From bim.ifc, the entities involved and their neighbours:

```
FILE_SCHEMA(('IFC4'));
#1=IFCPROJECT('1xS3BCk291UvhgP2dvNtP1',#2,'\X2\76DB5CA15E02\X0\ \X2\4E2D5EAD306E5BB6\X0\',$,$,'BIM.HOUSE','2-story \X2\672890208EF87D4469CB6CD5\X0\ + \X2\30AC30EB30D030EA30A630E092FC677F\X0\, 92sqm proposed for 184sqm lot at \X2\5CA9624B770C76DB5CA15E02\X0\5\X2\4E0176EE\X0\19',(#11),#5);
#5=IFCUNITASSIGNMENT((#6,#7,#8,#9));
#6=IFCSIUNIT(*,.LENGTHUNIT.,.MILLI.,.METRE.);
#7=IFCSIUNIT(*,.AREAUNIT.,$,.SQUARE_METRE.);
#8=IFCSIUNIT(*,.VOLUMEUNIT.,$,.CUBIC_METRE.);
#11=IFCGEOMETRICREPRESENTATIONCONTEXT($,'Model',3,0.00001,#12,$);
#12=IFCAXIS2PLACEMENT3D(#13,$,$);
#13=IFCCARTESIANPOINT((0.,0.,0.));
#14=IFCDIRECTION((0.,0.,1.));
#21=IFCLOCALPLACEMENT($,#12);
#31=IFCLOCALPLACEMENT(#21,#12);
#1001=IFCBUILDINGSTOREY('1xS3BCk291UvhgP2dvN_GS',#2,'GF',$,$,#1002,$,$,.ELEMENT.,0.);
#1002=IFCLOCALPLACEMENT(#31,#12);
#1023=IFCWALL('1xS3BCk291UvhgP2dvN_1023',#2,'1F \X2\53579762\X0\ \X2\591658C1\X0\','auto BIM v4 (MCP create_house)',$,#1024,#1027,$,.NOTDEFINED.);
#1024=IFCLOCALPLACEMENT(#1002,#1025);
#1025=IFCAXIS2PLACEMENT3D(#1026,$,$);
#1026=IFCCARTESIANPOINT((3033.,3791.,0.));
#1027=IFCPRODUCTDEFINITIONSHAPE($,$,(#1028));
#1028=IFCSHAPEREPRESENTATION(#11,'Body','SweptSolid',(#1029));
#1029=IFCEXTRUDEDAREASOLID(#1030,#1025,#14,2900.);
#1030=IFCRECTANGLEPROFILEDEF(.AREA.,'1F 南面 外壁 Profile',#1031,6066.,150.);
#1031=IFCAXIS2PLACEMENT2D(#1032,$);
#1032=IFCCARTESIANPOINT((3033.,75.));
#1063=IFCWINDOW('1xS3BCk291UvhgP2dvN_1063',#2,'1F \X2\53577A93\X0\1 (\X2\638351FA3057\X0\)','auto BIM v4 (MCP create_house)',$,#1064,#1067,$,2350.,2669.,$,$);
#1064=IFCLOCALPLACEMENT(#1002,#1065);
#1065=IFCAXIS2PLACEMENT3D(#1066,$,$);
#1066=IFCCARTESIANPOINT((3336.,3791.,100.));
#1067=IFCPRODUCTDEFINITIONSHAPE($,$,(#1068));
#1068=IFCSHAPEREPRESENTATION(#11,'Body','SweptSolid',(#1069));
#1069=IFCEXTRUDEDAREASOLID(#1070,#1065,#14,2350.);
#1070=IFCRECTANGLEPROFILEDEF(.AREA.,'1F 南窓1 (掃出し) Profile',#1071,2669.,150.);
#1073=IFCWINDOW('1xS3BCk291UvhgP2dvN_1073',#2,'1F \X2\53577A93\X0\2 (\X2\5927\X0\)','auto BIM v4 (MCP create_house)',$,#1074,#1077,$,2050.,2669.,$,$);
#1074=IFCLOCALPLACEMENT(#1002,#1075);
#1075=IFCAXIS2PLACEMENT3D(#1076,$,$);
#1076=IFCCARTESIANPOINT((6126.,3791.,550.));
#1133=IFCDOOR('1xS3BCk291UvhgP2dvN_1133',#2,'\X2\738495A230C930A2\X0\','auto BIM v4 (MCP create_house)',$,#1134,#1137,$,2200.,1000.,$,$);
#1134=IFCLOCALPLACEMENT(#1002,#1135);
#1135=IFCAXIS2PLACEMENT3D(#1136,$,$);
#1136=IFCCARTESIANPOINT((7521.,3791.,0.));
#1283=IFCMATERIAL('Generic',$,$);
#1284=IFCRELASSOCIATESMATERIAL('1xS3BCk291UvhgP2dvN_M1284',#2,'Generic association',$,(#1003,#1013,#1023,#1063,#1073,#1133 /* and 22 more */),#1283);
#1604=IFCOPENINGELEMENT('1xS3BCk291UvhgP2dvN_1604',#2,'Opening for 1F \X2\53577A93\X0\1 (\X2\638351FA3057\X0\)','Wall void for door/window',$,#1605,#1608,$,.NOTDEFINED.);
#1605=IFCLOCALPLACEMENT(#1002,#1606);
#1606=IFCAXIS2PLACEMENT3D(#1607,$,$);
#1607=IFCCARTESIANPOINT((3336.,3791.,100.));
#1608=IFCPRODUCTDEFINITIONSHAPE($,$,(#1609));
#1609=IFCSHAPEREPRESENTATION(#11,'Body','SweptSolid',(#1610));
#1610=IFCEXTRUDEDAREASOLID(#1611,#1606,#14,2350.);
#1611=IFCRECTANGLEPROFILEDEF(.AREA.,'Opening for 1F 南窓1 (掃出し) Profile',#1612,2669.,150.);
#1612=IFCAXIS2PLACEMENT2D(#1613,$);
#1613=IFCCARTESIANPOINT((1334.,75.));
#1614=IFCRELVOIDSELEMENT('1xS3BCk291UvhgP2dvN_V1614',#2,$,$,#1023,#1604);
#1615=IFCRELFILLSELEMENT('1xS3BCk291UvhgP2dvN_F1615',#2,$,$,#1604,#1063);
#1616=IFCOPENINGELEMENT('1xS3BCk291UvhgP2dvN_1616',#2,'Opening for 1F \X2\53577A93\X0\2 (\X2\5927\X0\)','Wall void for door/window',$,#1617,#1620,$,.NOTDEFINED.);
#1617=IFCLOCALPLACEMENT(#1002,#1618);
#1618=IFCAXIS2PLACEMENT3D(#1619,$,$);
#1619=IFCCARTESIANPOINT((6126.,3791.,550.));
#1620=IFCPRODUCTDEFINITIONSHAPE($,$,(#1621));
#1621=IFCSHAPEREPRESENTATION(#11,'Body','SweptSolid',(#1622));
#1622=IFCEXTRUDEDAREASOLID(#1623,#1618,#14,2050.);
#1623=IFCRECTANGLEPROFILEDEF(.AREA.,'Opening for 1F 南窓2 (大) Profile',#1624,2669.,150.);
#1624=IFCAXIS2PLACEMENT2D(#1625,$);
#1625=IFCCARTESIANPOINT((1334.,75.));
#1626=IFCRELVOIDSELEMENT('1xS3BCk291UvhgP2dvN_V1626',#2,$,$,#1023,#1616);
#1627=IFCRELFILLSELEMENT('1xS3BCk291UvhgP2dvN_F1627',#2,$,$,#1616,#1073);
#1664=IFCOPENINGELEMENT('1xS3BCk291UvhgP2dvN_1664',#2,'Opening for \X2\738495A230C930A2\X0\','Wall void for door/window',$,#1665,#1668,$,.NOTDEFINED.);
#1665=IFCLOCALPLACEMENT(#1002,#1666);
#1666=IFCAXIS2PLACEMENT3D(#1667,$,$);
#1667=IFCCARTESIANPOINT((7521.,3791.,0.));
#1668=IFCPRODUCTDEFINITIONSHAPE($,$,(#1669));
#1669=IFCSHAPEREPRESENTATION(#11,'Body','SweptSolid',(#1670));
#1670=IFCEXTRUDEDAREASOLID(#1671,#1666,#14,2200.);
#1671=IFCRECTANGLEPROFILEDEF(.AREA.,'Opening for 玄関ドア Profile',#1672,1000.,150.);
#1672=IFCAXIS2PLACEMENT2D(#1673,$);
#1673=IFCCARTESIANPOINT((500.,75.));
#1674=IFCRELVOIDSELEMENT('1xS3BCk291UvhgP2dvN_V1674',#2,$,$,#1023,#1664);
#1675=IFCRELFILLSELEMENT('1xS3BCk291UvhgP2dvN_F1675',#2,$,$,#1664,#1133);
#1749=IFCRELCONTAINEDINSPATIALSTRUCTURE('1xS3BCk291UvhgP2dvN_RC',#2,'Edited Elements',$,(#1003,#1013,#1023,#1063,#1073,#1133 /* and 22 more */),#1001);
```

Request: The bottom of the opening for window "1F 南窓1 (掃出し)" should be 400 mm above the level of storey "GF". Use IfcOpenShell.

```python
import numpy as np
import ifcopenshell
import ifcopenshell.api.geometry
import ifcopenshell.geom
import ifcopenshell.util.element
import ifcopenshell.util.placement
import ifcopenshell.util.shape
import ifcopenshell.util.unit

model = ifcopenshell.open("bim.ifc")
unit_scale = ifcopenshell.util.unit.calculate_unit_scale(model)

window = model.by_guid("1xS3BCk291UvhgP2dvN_1063")
opening = window.FillsVoids[0].RelatingOpeningElement
storey = ifcopenshell.util.element.get_container(window, ifc_class="IfcBuildingStorey")
level = ifcopenshell.util.placement.get_local_placement(storey.ObjectPlacement)[2, 3]

# The opening's origin need not be at the sill, so measure its lowest point.
shape = ifcopenshell.geom.create_shape(ifcopenshell.geom.settings(), opening)
bottom = ifcopenshell.util.shape.get_shape_bottom_elevation(shape, shape.geometry) / unit_scale
dz = level + 0.4 / unit_scale - bottom

shift = np.array([0.0, 0.0, dz])
# The window is not placed relative to its opening, so move both.
for product in (opening, window):
    matrix = ifcopenshell.util.placement.get_local_placement(product.ObjectPlacement)
    matrix[:3, 3] += shift
    ifcopenshell.api.geometry.edit_object_placement(model, product=product, matrix=matrix, is_si=False)

print(f"moved by {dz * unit_scale:+.3f} m")

model.write("bim_rev.ifc")
```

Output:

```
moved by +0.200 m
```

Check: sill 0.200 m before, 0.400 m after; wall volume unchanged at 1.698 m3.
